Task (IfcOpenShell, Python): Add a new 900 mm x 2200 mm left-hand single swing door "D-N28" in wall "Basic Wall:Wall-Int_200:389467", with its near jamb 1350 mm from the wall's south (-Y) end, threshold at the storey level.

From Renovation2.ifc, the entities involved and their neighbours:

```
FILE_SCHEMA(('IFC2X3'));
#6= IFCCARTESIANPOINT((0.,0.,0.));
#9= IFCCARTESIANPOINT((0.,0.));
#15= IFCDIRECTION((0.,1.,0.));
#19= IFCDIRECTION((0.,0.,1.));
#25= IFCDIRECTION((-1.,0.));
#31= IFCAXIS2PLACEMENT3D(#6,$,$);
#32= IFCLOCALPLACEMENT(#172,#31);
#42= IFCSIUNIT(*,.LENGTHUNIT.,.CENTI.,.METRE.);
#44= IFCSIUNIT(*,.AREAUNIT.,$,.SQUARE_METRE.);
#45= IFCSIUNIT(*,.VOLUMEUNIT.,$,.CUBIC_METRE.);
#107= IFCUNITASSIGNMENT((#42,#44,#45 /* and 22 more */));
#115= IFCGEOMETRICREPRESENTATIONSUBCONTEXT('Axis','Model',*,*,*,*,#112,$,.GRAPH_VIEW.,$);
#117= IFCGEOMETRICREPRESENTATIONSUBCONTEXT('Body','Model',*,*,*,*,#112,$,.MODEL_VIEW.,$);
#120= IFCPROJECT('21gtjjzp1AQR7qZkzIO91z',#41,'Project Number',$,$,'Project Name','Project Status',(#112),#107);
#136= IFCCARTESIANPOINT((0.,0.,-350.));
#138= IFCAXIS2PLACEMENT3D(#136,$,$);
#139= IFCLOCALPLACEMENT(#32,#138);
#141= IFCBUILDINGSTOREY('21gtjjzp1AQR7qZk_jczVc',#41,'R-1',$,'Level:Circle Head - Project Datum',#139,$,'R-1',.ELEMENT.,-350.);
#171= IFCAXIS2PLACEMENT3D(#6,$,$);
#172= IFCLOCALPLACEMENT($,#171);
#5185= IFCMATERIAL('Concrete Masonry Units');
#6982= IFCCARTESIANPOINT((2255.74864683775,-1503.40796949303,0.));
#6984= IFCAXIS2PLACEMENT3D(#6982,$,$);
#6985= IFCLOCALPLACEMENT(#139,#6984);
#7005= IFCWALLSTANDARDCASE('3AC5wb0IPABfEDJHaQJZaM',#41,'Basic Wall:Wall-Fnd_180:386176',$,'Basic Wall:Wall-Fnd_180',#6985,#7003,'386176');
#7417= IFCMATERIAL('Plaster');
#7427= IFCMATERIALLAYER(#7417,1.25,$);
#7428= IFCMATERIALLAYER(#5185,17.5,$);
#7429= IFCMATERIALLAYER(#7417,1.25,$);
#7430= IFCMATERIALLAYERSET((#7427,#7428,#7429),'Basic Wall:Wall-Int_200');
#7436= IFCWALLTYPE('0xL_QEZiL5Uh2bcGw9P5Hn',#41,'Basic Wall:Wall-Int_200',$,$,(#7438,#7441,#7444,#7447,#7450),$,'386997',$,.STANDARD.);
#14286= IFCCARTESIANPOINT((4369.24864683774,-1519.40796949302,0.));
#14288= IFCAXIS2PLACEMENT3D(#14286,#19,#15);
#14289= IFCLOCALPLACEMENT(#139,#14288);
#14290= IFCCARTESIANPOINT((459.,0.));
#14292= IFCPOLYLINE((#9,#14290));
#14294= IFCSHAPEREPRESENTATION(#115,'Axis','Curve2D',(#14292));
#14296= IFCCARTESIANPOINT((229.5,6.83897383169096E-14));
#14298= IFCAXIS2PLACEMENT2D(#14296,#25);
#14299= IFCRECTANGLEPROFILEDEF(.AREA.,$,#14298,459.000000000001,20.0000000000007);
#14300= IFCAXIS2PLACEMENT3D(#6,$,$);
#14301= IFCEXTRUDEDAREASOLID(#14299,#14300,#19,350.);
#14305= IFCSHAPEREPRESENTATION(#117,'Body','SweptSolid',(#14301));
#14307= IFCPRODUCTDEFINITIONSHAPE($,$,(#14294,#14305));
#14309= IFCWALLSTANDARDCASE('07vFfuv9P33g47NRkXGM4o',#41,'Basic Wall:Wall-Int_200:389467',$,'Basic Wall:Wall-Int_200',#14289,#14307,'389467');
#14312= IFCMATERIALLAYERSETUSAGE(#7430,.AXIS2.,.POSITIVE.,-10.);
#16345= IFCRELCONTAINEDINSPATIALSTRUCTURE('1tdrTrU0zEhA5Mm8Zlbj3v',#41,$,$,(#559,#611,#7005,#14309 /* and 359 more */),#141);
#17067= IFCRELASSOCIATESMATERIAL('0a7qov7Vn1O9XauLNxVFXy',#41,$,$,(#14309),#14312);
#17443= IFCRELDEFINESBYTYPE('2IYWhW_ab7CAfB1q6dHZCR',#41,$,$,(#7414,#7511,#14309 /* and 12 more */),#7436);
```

```python
import numpy as np
import ifcopenshell
import ifcopenshell.api.feature
import ifcopenshell.api.geometry
import ifcopenshell.api.root
import ifcopenshell.api.spatial
import ifcopenshell.api.type
import ifcopenshell.geom
import ifcopenshell.util.element
import ifcopenshell.util.placement
import ifcopenshell.util.representation
import ifcopenshell.util.shape
import ifcopenshell.util.unit

model = ifcopenshell.open("Renovation2.ifc")
unit_scale = ifcopenshell.util.unit.calculate_unit_scale(model)
settings = ifcopenshell.geom.settings()


def volume(element):
    """Net volume in cubic metres, openings subtracted."""
    shape = ifcopenshell.geom.create_shape(settings, element)
    return ifcopenshell.util.shape.get_volume(shape.geometry)


wall = model.by_guid("07vFfuv9P33g47NRkXGM4o")
storey = ifcopenshell.util.element.get_container(wall, ifc_class="IfcBuildingStorey")
context = ifcopenshell.util.representation.get_context(model, "Model", "Body", "MODEL_VIEW")
before = volume(wall)

width, height, from_end, sill = 0.9, 2.2, 1.35, 0.0  # metres

# The wall runs along its own X axis, and the end named is its -X end.
wall_shape = ifcopenshell.geom.create_shape(settings, wall)
x, y, z = ifcopenshell.util.shape.get_vertices(wall_shape.geometry).T
start = x.min() + from_end
face, thickness = float(y.min()), float(y.max() - y.min())
wall_matrix = ifcopenshell.util.placement.get_local_placement(wall.ObjectPlacement)
level = ifcopenshell.util.placement.get_local_placement(storey.ObjectPlacement)[2, 3]


def in_wall(x, y):
    """Placement at x, y metres in the wall's axes, at sill height."""
    matrix = wall_matrix.copy()
    matrix[:, 3] = wall_matrix @ np.array([x / unit_scale, y / unit_scale, 0.0, 1.0])
    matrix[2, 3] = level + sill / unit_scale
    return matrix


# Opening: a box that overshoots both wall faces by 50 mm.
opening = ifcopenshell.api.root.create_entity(model, ifc_class="IfcOpeningElement")
box = ifcopenshell.api.geometry.add_wall_representation(
    model, context=context, length=width, height=height, thickness=thickness + 0.1
)
ifcopenshell.api.geometry.assign_representation(model, product=opening, representation=box)
ifcopenshell.api.geometry.edit_object_placement(model, product=opening, matrix=in_wall(start, face - 0.05), is_si=False)
ifcopenshell.api.feature.add_feature(model, feature=opening, element=wall)

door = ifcopenshell.api.root.create_entity(model, ifc_class="IfcDoor", name="D-N28")
door.OverallWidth, door.OverallHeight = width / unit_scale, height / unit_scale
body = ifcopenshell.api.geometry.add_door_representation(
    model,
    context=context,
    overall_width=door.OverallWidth,
    overall_height=door.OverallHeight,
    operation_type="SINGLE_SWING_LEFT",
    lining_properties={"LiningDepth": thickness / unit_scale, "ThresholdDepth": thickness / unit_scale},
)
ifcopenshell.api.geometry.assign_representation(model, product=door, representation=body)
ifcopenshell.api.spatial.assign_container(model, products=[door], relating_structure=storey)
fills = ifcopenshell.api.feature.add_filling(model, opening=opening, element=door)
fills.OwnerHistory = door.OwnerHistory  # required in IFC2X3

# IFC2X3 keeps the operation on the door style.
style = ifcopenshell.api.root.create_entity(model, ifc_class="IfcDoorStyle", name="D-N28")
style.OperationType, style.ConstructionType = "SINGLE_SWING_LEFT", "NOTDEFINED"
style.ParameterTakesPrecedence = style.Sizeable = False
ifcopenshell.api.type.assign_type(model, related_objects=[door], relating_type=style)

# The lining spans the wall, so the door starts at the wall face.
ifcopenshell.api.geometry.edit_object_placement(model, product=door, matrix=in_wall(start, face), is_si=False)

after = volume(wall)

print(f"wall volume {before:.3f} -> {after:.3f} m3")

model.write("Renovation2_edited.ifc")
```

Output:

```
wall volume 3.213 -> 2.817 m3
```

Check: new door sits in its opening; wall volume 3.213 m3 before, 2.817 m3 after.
